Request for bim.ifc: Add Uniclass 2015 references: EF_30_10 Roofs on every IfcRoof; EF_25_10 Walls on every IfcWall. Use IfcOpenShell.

First a look at what the model holds.

```python
import ifcopenshell

model = ifcopenshell.open("bim.ifc")
print(model.schema)
print("classifications:", [c.Name for c in model.by_type("IfcClassification")])
for ifc_class in ("IfcDoor", "IfcRoof", "IfcStair", "IfcWall", "IfcWindow"):
    print(ifc_class, len(model.by_type(ifc_class)))
```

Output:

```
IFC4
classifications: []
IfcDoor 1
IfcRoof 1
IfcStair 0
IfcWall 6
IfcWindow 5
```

```python
import ifcopenshell
import ifcopenshell.api.classification

model = ifcopenshell.open("bim.ifc")

system = ifcopenshell.api.classification.add_classification(model, classification="Uniclass 2015")

codes = {
    "IfcRoof": ("EF_30_10", "Roofs"),
    "IfcWall": ("EF_25_10", "Walls"),
}
for ifc_class, (code, name) in codes.items():
    products = model.by_type(ifc_class)
    ifcopenshell.api.classification.add_reference(
        model, products=products, classification=system, identification=code, name=name
    )
    print(code, len(products))

model.write("bim_rev.ifc")
```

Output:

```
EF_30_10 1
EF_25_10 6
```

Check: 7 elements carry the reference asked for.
